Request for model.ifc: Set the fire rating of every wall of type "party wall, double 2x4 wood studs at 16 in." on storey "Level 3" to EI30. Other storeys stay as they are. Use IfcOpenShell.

First a look at what the model holds.

```python
import ifcopenshell
import ifcopenshell.util.element

model = ifcopenshell.open("model.ifc")
print(model.schema)
storey = next(s for s in model.by_type("IfcBuildingStorey") if s.Name == "Level 3")
walls = [e for e in ifcopenshell.util.element.get_decomposition(storey) if e.is_a("IfcWall")]
seen = {}
for e in walls:
    element_type = ifcopenshell.util.element.get_type(e)
    key = (element_type.Name if element_type != e and element_type else None, ifcopenshell.util.element.get_pset(e, "Pset_WallCommon", "FireRating"))
    seen[key] = seen.get(key, 0) + 1
for (name, value), count in sorted(seen.items(), key=str):
    print(count, "x", name, "|", value)
```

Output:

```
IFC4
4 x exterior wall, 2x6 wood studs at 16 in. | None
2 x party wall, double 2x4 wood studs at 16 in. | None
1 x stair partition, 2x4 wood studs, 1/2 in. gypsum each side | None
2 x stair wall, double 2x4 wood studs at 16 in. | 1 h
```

```python
import ifcopenshell
import ifcopenshell.api.pset
import ifcopenshell.util.element

model = ifcopenshell.open("model.ifc")

storey = next(s for s in model.by_type("IfcBuildingStorey") if s.Name == "Level 3")
walls = [e for e in ifcopenshell.util.element.get_decomposition(storey) if e.is_a("IfcWall")]

count = 0
for e in walls:
    element_type = ifcopenshell.util.element.get_type(e)
    if element_type in (None, e) or element_type.Name != "party wall, double 2x4 wood studs at 16 in.":
        continue
    # add_pset returns the element's existing set when there is one.
    pset = ifcopenshell.api.pset.add_pset(model, product=e, name="Pset_WallCommon")
    ifcopenshell.api.pset.edit_pset(model, pset=pset, properties={"FireRating": "EI30"})
    count += 1

print(count, "walls updated")

model.write("model-out.ifc")
```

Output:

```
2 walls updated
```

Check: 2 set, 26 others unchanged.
